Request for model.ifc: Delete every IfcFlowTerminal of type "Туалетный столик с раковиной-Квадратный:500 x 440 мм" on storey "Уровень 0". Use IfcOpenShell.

First a look at what the model holds.

```python
import ifcopenshell
import ifcopenshell.util.element

model = ifcopenshell.open("model.ifc")
print(model.schema)
storey = next(s for s in model.by_type("IfcBuildingStorey") if s.Name == "Уровень 0")
terminals = [e for e in ifcopenshell.util.element.get_decomposition(storey) if e.is_a("IfcFlowTerminal")]
seen = {}
for e in terminals:
    element_type = ifcopenshell.util.element.get_type(e)
    name = element_type.Name if element_type not in (None, e) else None
    seen[name] = seen.get(name, 0) + 1
for name, count in sorted(seen.items(), key=str):
    print(count, "x", name)
```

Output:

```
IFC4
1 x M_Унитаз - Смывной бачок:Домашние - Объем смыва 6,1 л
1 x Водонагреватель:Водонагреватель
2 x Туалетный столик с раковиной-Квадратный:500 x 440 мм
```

```python
import ifcopenshell
import ifcopenshell.api.root
import ifcopenshell.util.element

model = ifcopenshell.open("model.ifc")

storey = next(s for s in model.by_type("IfcBuildingStorey") if s.Name == "Уровень 0")
terminals = [e for e in ifcopenshell.util.element.get_decomposition(storey) if e.is_a("IfcFlowTerminal")]
targets = [e for e in terminals if (t := ifcopenshell.util.element.get_type(e)) not in (None, e) and t.Name == "Туалетный столик с раковиной-Квадратный:500 x 440 мм"]

for e in targets:
    ifcopenshell.api.root.remove_product(model, product=e)
print(len(targets), "removed")

model.write("model_updated.ifc")
```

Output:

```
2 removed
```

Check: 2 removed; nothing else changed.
